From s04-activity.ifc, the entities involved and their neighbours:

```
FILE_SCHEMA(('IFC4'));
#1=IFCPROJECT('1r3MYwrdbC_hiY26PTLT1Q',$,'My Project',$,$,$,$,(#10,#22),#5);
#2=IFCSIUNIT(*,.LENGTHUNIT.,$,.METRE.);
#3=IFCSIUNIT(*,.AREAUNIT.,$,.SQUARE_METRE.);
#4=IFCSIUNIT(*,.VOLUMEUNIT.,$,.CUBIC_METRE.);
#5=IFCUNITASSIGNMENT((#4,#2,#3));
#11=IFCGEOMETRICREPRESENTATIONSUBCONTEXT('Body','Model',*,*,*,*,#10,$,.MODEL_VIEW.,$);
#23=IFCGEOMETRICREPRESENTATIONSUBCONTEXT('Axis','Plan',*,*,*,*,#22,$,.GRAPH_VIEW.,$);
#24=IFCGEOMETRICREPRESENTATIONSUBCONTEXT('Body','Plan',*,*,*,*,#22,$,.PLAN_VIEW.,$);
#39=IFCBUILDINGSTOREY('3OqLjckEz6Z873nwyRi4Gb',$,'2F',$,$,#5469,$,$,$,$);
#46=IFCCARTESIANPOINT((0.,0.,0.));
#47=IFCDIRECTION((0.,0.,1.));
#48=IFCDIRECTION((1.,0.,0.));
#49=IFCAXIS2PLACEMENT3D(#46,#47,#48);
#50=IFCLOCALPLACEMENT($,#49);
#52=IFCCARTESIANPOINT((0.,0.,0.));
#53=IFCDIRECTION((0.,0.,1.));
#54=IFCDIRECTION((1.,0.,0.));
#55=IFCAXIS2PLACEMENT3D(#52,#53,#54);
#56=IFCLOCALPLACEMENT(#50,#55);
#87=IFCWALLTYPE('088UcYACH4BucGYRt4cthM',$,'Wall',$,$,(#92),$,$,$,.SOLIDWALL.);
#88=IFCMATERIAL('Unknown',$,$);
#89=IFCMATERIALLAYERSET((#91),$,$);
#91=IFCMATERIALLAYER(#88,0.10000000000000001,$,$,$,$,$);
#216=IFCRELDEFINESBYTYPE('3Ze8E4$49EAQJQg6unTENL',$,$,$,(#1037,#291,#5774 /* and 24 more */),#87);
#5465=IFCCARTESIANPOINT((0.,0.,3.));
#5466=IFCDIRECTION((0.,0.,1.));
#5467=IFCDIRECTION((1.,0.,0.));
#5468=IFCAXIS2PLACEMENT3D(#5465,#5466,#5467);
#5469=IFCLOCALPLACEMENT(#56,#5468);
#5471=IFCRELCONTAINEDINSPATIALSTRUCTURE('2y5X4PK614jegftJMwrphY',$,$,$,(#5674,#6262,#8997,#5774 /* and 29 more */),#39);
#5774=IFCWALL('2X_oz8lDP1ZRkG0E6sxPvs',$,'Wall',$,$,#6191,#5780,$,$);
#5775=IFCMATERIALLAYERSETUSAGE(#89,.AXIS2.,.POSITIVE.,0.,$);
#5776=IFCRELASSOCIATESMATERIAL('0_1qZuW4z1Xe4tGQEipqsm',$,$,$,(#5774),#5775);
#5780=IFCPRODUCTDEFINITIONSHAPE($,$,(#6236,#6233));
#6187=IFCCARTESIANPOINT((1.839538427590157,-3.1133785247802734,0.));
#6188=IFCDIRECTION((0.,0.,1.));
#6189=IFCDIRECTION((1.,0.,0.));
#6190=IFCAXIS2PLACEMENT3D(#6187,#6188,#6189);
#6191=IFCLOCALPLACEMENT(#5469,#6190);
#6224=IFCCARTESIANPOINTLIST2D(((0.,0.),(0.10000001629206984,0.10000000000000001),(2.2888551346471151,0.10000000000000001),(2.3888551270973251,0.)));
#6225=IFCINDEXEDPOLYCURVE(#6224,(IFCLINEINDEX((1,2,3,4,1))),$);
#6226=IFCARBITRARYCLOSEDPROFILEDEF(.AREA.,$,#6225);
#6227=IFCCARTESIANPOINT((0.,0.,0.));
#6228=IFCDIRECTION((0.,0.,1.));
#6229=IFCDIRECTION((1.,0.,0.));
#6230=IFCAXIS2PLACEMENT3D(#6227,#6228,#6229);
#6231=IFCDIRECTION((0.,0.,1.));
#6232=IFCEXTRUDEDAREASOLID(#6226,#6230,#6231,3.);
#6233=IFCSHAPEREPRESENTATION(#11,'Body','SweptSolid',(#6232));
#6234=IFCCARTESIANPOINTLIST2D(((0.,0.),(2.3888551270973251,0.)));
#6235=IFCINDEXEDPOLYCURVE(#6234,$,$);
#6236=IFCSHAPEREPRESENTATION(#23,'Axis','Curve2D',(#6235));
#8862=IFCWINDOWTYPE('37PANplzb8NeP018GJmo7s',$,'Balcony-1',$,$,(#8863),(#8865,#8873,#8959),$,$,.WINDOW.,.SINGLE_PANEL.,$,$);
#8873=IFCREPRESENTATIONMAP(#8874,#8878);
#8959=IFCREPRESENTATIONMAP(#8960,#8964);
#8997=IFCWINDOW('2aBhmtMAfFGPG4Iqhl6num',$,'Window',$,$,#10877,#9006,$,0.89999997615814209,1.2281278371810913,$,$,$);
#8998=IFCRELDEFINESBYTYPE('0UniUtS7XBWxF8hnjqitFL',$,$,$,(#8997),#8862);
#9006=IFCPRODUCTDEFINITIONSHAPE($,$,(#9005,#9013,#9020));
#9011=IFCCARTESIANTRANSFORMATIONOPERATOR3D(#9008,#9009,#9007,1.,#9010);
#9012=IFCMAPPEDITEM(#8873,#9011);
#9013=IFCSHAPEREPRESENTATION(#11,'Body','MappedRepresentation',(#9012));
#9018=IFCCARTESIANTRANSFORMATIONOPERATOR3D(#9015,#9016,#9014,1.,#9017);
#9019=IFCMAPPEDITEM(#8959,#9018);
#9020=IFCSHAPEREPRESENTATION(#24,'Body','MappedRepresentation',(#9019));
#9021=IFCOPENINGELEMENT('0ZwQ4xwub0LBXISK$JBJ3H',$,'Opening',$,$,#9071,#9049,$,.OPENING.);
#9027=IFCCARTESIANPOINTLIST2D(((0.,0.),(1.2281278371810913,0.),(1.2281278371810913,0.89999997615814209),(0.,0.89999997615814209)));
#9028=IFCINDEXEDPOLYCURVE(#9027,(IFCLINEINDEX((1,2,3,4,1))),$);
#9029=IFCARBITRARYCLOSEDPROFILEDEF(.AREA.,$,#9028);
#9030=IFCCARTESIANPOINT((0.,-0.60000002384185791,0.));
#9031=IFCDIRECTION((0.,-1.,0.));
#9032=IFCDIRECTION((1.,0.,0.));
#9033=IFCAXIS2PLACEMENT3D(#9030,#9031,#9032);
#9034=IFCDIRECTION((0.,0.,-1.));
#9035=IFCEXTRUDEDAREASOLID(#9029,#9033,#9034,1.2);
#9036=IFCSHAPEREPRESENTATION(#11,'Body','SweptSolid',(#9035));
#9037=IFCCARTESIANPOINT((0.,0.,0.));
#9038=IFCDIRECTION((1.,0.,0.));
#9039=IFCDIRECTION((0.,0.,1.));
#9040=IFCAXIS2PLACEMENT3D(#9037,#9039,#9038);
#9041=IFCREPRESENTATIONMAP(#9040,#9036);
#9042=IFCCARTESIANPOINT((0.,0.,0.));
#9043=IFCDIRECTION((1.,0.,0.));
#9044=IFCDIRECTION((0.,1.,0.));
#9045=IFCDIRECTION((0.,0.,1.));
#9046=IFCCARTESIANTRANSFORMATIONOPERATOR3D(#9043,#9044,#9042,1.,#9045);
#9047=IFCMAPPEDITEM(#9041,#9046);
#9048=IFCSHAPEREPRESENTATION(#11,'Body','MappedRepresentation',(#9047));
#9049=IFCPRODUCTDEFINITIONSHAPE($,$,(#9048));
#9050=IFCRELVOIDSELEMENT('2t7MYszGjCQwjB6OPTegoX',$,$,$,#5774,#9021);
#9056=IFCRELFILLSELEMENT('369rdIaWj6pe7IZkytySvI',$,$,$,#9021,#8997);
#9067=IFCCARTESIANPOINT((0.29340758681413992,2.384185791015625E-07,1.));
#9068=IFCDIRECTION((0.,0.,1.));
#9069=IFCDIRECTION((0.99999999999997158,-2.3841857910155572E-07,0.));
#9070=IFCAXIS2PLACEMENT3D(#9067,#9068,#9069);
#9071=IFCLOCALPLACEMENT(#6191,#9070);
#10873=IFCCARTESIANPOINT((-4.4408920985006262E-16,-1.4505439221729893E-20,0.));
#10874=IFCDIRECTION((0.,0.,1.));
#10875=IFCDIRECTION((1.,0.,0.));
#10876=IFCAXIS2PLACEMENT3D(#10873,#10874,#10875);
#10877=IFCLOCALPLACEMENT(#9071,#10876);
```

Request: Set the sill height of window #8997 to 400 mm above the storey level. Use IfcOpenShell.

```python
import numpy as np
import ifcopenshell
import ifcopenshell.api.geometry
import ifcopenshell.geom
import ifcopenshell.util.element
import ifcopenshell.util.placement
import ifcopenshell.util.shape
import ifcopenshell.util.unit

model = ifcopenshell.open("s04-activity.ifc")
unit_scale = ifcopenshell.util.unit.calculate_unit_scale(model)

window = model.by_id(8997)
opening = window.FillsVoids[0].RelatingOpeningElement
storey = ifcopenshell.util.element.get_container(window, ifc_class="IfcBuildingStorey")
level = ifcopenshell.util.placement.get_local_placement(storey.ObjectPlacement)[2, 3]

# The opening's origin need not be at the sill, so measure its lowest point.
shape = ifcopenshell.geom.create_shape(ifcopenshell.geom.settings(), opening)
bottom = ifcopenshell.util.shape.get_shape_bottom_elevation(shape, shape.geometry) / unit_scale
dz = level + 0.4 / unit_scale - bottom

shift = np.array([0.0, 0.0, dz])
# The window is placed relative to its opening, so it follows when the opening moves.
matrix = ifcopenshell.util.placement.get_local_placement(opening.ObjectPlacement)
matrix[:3, 3] += shift
ifcopenshell.api.geometry.edit_object_placement(
    model, product=opening, matrix=matrix, is_si=False, should_transform_children=True
)

print(f"moved by {dz * unit_scale:+.3f} m")

model.write("s04-activity_v2.ifc")
```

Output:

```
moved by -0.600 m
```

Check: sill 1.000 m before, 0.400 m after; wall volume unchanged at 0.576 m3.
